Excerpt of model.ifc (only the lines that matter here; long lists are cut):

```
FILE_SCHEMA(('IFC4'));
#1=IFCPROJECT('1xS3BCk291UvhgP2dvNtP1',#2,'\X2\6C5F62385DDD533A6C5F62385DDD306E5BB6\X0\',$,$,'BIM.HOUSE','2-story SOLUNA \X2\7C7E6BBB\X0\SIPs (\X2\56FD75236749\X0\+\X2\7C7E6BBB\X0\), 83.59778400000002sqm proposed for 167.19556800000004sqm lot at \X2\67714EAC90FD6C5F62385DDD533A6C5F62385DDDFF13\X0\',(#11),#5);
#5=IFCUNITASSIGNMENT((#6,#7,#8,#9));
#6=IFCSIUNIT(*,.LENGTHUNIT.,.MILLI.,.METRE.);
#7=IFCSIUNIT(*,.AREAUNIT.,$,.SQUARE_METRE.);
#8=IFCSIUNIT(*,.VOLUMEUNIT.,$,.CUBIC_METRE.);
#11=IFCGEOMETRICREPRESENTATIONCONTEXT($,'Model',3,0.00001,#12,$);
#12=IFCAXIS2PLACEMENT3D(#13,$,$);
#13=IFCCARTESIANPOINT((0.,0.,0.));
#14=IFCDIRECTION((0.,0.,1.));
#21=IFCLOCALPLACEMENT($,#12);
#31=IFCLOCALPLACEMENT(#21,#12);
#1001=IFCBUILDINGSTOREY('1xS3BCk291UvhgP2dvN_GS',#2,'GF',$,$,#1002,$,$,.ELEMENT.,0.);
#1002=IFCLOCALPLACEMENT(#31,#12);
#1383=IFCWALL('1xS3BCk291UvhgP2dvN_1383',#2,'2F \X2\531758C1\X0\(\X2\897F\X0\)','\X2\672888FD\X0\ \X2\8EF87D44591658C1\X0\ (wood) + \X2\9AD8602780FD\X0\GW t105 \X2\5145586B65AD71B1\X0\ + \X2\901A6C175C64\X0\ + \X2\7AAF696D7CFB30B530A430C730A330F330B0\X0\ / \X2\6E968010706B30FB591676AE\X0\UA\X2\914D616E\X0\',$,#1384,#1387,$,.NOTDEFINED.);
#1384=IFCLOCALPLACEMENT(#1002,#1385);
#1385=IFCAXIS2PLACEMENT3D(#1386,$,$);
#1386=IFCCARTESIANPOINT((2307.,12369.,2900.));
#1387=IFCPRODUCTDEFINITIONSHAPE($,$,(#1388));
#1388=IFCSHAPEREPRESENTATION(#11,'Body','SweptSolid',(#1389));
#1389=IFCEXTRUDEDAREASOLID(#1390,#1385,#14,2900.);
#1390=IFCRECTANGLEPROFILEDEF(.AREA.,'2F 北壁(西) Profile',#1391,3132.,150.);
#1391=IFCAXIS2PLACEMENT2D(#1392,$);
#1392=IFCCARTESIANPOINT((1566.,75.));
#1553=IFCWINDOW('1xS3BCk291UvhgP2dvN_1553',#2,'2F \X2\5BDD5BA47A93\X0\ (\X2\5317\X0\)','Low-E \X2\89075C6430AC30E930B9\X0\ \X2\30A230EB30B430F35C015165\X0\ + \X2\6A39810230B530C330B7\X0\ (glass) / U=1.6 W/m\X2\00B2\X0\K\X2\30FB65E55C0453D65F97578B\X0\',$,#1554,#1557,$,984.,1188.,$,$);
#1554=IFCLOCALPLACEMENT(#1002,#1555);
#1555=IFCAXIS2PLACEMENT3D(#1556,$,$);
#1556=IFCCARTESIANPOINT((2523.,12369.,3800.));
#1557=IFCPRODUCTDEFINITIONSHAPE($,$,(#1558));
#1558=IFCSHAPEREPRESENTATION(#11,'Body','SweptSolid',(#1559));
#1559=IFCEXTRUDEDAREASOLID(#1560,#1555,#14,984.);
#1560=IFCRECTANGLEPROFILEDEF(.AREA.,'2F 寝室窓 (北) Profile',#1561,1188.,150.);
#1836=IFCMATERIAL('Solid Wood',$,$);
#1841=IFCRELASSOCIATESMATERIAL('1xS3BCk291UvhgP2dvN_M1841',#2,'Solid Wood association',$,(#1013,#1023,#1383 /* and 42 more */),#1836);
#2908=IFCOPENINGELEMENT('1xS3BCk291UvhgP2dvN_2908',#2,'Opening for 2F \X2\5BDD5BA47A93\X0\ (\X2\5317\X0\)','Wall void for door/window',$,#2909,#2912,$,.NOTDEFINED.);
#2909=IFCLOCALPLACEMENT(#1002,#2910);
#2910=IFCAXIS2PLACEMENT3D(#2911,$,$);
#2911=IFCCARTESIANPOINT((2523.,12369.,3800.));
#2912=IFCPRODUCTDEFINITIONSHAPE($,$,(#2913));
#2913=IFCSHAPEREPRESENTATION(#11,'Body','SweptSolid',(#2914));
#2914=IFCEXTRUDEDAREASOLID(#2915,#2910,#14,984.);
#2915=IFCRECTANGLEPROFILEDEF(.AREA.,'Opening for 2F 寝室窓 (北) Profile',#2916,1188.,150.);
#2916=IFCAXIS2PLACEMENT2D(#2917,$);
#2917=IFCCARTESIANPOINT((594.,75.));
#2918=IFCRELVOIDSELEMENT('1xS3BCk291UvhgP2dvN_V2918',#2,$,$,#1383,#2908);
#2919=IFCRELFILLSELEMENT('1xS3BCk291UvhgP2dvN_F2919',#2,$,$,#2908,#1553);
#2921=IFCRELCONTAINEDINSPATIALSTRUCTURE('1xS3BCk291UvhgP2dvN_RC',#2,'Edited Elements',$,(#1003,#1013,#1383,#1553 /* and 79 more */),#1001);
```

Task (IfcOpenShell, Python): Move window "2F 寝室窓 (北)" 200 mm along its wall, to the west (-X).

```python
import ifcopenshell
import ifcopenshell.api.geometry
import ifcopenshell.util.placement

model = ifcopenshell.open("model.ifc")

window = model.by_guid("1xS3BCk291UvhgP2dvN_1553")
opening = window.FillsVoids[0].RelatingOpeningElement
wall = opening.VoidsElements[0].RelatingBuildingElement

wall_matrix = ifcopenshell.util.placement.get_local_placement(wall.ObjectPlacement)
shift = wall_matrix[:3, 0] * -200.0
before = ifcopenshell.util.placement.get_local_placement(window.ObjectPlacement)[:3, 3].copy()

# The window is not placed relative to its opening, so move both.
for product in (opening, window):
    matrix = ifcopenshell.util.placement.get_local_placement(product.ObjectPlacement)
    matrix[:3, 3] += shift
    ifcopenshell.api.geometry.edit_object_placement(model, product=product, matrix=matrix, is_si=False)

after = ifcopenshell.util.placement.get_local_placement(window.ObjectPlacement)[:3, 3]
print("window moved by", (after - before).round(3) + 0.0)

model.write("model_updated.ifc")
```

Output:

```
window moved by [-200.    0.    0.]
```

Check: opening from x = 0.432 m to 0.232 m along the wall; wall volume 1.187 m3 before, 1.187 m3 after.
